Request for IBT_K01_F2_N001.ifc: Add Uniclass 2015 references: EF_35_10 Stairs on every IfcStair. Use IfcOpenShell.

First a look at what the model holds.

```python
import ifcopenshell

model = ifcopenshell.open("IBT_K01_F2_N001.ifc")
print(model.schema)
print("classifications:", [c.Name for c in model.by_type("IfcClassification")])
for ifc_class in ("IfcDoor", "IfcRoof", "IfcStair", "IfcWall", "IfcWindow"):
    print(ifc_class, len(model.by_type(ifc_class)))
```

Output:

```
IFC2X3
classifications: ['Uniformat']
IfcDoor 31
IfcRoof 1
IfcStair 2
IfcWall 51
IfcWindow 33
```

```python
import ifcopenshell
import ifcopenshell.api.classification

model = ifcopenshell.open("IBT_K01_F2_N001.ifc")

# IFC2X3 requires Source and Edition and has no link from the project to the system.
system = model.create_entity("IfcClassification", Source="NBS", Edition="2015", Name="Uniclass 2015")

codes = {
    "IfcStair": ("EF_35_10", "Stairs"),
}
for ifc_class, (code, name) in codes.items():
    products = model.by_type(ifc_class)
    ifcopenshell.api.classification.add_reference(
        model, products=products, classification=system, identification=code, name=name
    )
    print(code, len(products))

model.write("IBT_K01_F2_N001_edited.ifc")
```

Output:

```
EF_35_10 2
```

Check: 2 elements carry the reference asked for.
